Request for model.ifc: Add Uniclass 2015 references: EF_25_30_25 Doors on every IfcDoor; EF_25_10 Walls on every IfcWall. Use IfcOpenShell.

First a look at what the model holds.

```python
import ifcopenshell

model = ifcopenshell.open("model.ifc")
print(model.schema)
print("classifications:", [c.Name for c in model.by_type("IfcClassification")])
for ifc_class in ("IfcDoor", "IfcRoof", "IfcStair", "IfcWall", "IfcWindow"):
    print(ifc_class, len(model.by_type(ifc_class)))
```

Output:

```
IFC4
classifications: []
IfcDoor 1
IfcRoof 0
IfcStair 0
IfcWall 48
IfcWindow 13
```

```python
import ifcopenshell
import ifcopenshell.api.classification

model = ifcopenshell.open("model.ifc")

system = ifcopenshell.api.classification.add_classification(model, classification="Uniclass 2015")

codes = {
    "IfcDoor": ("EF_25_30_25", "Doors"),
    "IfcWall": ("EF_25_10", "Walls"),
}
for ifc_class, (code, name) in codes.items():
    products = model.by_type(ifc_class)
    ifcopenshell.api.classification.add_reference(
        model, products=products, classification=system, identification=code, name=name
    )
    print(code, len(products))

model.write("model_rev.ifc")
```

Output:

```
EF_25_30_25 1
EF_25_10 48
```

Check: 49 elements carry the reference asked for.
